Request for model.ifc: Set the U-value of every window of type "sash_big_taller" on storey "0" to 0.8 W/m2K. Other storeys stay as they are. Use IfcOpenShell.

First a look at what the model holds.

```python
import ifcopenshell
import ifcopenshell.util.element

model = ifcopenshell.open("model.ifc")
print(model.schema)
storey = next(s for s in model.by_type("IfcBuildingStorey") if s.Name == "0")
windows = [e for e in ifcopenshell.util.element.get_decomposition(storey) if e.is_a("IfcWindow")]
seen = {}
for e in windows:
    element_type = ifcopenshell.util.element.get_type(e)
    key = (element_type.Name if element_type != e and element_type else None, ifcopenshell.util.element.get_pset(e, "Pset_WindowCommon", "ThermalTransmittance"))
    seen[key] = seen.get(key, 0) + 1
for (name, value), count in sorted(seen.items(), key=str):
    print(count, "x", name, "|", value)
```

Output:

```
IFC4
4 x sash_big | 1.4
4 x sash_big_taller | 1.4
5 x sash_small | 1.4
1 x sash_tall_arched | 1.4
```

```python
import ifcopenshell
import ifcopenshell.api.pset
import ifcopenshell.util.element

model = ifcopenshell.open("model.ifc")

storey = next(s for s in model.by_type("IfcBuildingStorey") if s.Name == "0")
windows = [e for e in ifcopenshell.util.element.get_decomposition(storey) if e.is_a("IfcWindow")]

count = 0
for e in windows:
    element_type = ifcopenshell.util.element.get_type(e)
    if element_type in (None, e) or element_type.Name != "sash_big_taller":
        continue
    # add_pset returns the element's existing set when there is one.
    pset = ifcopenshell.api.pset.add_pset(model, product=e, name="Pset_WindowCommon")
    ifcopenshell.api.pset.edit_pset(model, pset=pset, properties={"ThermalTransmittance": 0.8})
    count += 1

print(count, "windows updated")

model.write("model_rev.ifc")
```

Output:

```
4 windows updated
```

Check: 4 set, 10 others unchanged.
